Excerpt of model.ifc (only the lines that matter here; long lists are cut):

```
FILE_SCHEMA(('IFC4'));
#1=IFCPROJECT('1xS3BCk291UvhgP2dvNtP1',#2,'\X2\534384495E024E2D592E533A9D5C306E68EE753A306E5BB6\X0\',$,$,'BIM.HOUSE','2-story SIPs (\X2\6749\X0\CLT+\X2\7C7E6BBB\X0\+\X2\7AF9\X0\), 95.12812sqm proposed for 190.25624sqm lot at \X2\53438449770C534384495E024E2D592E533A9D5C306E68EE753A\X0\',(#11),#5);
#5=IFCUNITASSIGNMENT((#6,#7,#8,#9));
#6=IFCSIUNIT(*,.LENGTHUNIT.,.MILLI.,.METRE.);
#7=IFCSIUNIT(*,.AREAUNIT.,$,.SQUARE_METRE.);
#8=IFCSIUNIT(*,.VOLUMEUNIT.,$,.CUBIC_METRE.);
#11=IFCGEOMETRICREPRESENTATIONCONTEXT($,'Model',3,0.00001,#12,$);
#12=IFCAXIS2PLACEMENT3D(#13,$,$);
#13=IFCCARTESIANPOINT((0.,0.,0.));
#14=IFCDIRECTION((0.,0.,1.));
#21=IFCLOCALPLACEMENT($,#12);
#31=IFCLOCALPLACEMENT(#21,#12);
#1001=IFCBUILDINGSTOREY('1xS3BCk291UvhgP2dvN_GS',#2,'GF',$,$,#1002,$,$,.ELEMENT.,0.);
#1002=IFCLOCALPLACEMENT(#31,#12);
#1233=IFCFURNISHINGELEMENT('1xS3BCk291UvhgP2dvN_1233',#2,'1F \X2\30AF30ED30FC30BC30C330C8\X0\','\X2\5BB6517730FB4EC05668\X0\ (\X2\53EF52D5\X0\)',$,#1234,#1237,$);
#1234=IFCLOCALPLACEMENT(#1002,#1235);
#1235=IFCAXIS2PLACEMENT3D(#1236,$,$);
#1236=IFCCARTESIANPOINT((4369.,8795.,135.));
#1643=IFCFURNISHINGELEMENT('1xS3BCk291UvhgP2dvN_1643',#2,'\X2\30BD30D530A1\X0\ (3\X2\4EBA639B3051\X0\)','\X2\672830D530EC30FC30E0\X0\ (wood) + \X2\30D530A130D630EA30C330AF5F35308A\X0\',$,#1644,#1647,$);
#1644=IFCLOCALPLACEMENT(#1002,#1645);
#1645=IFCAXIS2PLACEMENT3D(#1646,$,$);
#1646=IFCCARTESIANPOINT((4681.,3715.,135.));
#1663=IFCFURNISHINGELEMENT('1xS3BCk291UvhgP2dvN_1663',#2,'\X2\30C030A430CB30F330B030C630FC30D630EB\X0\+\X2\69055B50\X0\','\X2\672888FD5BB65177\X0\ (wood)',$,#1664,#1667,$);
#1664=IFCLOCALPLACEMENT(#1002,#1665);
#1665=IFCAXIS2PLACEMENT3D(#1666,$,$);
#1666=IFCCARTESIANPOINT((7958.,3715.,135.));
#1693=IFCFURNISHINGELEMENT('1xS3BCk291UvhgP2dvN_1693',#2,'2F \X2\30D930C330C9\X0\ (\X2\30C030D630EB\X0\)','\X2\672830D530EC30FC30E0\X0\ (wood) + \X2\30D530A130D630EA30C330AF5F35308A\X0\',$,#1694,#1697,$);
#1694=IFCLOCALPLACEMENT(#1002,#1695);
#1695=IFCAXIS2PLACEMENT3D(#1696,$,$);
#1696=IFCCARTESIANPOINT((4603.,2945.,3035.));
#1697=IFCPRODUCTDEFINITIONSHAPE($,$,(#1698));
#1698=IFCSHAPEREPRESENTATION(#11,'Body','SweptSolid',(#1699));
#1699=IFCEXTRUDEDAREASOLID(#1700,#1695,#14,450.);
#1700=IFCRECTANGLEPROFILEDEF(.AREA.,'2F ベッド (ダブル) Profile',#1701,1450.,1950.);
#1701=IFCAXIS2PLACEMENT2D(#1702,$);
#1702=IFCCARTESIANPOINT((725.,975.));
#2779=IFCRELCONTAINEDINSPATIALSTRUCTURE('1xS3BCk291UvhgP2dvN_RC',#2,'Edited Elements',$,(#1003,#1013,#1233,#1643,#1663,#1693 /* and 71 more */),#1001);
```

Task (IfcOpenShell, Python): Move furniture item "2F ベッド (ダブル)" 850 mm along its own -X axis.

```python
import ifcopenshell
import ifcopenshell.api.geometry
import ifcopenshell.util.placement
import ifcopenshell.util.unit

model = ifcopenshell.open("model.ifc")
unit_scale = ifcopenshell.util.unit.calculate_unit_scale(model)

item = model.by_guid("1xS3BCk291UvhgP2dvN_1693")
matrix = ifcopenshell.util.placement.get_local_placement(item.ObjectPlacement)
matrix[:3, 3] -= matrix[:3, 0] * 0.85 / unit_scale
ifcopenshell.api.geometry.edit_object_placement(model, product=item, matrix=matrix, is_si=False)

print(ifcopenshell.util.placement.get_local_placement(item.ObjectPlacement).round(3) + 0.0)

model.write("model-out.ifc")
```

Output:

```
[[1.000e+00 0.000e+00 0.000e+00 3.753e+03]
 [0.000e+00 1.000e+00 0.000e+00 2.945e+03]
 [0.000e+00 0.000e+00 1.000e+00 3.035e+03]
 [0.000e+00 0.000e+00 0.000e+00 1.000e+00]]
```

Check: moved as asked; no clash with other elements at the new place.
